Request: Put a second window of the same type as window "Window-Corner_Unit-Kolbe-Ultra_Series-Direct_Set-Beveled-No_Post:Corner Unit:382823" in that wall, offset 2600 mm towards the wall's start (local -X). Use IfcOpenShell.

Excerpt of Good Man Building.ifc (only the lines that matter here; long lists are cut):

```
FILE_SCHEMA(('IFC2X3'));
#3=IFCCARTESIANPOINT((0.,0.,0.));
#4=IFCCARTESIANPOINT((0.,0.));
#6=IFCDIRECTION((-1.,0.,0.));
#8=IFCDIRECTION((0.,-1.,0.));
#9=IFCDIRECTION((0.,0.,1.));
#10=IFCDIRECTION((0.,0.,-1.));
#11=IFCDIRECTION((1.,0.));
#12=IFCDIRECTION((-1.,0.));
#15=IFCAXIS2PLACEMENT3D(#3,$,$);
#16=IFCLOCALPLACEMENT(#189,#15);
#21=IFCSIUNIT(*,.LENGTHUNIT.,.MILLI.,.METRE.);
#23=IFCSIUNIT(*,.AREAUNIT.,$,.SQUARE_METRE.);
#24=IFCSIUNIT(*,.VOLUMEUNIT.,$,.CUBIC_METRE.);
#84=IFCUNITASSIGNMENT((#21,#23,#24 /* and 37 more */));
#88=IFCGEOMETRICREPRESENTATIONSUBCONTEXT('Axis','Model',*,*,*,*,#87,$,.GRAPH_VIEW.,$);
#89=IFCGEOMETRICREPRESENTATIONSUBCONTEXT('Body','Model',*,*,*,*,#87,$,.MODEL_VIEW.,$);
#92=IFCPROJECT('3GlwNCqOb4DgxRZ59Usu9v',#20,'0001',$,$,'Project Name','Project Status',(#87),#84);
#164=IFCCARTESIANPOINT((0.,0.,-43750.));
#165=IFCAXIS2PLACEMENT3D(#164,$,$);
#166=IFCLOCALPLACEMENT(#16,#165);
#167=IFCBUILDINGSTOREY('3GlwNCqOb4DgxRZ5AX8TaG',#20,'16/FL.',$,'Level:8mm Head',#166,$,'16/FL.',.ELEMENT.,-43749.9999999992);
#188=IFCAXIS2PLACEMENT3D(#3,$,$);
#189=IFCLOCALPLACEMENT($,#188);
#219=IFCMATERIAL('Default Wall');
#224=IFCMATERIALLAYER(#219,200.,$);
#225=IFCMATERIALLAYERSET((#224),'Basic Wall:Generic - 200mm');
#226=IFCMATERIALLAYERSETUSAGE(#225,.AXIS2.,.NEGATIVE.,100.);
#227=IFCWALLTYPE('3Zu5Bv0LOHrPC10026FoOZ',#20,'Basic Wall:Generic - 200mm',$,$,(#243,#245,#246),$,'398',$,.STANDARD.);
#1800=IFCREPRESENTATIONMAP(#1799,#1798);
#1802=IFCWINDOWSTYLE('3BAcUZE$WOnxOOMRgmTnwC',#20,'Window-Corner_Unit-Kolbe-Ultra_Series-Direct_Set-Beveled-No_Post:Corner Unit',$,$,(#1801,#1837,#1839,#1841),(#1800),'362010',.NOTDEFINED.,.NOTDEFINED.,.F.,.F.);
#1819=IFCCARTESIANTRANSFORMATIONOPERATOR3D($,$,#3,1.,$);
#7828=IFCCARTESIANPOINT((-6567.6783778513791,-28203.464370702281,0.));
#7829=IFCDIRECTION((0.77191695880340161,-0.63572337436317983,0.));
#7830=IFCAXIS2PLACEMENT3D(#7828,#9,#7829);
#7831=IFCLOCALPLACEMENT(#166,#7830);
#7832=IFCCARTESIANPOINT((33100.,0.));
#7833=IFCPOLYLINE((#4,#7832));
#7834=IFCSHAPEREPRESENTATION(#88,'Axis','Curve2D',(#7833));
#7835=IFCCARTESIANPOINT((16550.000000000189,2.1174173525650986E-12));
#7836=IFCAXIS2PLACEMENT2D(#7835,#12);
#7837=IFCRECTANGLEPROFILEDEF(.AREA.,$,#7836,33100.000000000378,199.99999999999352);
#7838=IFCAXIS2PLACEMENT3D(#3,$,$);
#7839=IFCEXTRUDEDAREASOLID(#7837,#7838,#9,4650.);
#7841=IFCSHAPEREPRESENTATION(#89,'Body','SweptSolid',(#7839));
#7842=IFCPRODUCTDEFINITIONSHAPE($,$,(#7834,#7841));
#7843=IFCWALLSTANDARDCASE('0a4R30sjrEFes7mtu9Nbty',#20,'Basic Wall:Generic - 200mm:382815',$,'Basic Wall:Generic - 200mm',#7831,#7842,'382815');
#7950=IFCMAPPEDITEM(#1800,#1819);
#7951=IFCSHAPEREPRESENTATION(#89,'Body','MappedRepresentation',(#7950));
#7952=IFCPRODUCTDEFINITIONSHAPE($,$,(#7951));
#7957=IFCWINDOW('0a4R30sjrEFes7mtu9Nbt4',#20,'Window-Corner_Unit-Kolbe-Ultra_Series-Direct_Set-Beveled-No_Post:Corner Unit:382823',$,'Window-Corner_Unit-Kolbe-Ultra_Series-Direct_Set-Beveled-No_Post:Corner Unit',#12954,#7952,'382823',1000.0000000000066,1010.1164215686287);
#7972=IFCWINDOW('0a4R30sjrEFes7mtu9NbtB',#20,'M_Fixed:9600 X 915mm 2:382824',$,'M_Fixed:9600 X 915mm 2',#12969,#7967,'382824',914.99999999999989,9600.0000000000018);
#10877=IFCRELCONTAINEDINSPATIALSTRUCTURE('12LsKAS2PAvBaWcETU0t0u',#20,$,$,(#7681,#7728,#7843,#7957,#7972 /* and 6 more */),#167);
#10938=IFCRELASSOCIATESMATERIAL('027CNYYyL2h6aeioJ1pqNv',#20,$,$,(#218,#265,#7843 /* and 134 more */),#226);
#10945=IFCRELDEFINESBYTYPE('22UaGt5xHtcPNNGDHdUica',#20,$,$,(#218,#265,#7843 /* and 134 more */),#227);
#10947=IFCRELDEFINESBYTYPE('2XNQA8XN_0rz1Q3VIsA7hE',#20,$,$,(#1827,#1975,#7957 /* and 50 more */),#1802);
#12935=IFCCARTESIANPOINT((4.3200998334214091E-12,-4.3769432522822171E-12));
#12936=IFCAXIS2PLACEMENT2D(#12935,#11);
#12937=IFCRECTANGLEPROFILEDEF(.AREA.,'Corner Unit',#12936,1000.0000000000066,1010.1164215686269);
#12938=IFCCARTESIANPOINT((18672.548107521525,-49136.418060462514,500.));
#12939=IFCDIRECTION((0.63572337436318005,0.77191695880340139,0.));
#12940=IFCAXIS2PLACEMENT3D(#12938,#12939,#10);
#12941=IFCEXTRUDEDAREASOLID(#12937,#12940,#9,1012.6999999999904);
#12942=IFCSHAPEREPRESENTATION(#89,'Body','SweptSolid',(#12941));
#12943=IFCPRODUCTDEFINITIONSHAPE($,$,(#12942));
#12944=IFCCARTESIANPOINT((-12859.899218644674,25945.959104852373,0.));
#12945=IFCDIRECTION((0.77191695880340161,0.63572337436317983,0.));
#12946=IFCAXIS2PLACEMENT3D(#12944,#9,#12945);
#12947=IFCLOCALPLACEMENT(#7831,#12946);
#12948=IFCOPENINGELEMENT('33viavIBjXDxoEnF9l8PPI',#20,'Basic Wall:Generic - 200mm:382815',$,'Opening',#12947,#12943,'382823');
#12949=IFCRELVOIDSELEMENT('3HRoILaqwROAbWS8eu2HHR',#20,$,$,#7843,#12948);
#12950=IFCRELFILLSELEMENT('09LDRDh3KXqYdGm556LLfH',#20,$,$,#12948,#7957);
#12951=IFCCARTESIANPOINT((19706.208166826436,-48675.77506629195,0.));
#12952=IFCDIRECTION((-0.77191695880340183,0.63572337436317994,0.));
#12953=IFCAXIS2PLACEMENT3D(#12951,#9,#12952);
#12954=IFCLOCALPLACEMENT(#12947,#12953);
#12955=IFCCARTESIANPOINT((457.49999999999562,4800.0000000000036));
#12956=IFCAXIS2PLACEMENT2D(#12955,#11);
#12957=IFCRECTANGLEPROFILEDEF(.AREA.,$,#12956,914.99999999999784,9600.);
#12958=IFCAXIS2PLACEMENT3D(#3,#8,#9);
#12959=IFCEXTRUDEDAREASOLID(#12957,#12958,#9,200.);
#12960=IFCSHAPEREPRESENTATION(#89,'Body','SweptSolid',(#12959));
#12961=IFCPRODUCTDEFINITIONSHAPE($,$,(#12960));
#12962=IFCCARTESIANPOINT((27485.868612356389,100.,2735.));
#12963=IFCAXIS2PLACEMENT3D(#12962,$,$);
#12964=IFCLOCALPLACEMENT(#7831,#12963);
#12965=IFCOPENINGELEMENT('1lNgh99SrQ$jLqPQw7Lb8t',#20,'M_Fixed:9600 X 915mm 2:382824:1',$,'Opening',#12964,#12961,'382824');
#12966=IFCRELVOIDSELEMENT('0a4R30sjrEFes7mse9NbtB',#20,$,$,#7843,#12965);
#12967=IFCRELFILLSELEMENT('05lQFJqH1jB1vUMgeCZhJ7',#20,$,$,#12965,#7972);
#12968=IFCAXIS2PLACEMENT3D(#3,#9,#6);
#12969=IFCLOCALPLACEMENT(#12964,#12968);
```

```python
import ifcopenshell
import ifcopenshell.api.feature
import ifcopenshell.api.geometry
import ifcopenshell.api.root
import ifcopenshell.geom
import ifcopenshell.util.element
import ifcopenshell.util.placement
import ifcopenshell.util.shape

model = ifcopenshell.open("Good Man Building.ifc")
settings = ifcopenshell.geom.settings()


def volume(element):
    """Net volume in cubic metres, openings subtracted."""
    shape = ifcopenshell.geom.create_shape(settings, element)
    return ifcopenshell.util.shape.get_volume(shape.geometry)


def reuse_history(source, copy):
    """copy_class also copies each property set's owner history, people and application; keep the originals."""
    for rel in copy.IsDefinedBy:
        if rel.is_a("IfcRelDefinesByProperties") and (history := rel.RelatingPropertyDefinition.OwnerHistory):
            rel.RelatingPropertyDefinition.OwnerHistory = source.OwnerHistory
            ifcopenshell.util.element.remove_deep2(model, history)


window = model.by_guid("0a4R30sjrEFes7mtu9Nbt4")
opening = window.FillsVoids[0].RelatingOpeningElement
wall = opening.VoidsElements[0].RelatingBuildingElement
before = volume(wall)
shift = ifcopenshell.util.placement.get_local_placement(wall.ObjectPlacement)[:3, 0] * -2600.0

# copy_class copies the void relationship, type, container and properties, but no geometry.
new_opening = ifcopenshell.api.root.copy_class(model, product=opening)
new_opening.Representation = ifcopenshell.util.element.copy_deep(
    model, opening.Representation, exclude=["IfcGeometricRepresentationContext", "IfcRepresentationMap"]
)
new_opening.Name = "Basic Wall:Generic - 200mm"
new_opening.Tag = None
new_window = ifcopenshell.api.root.copy_class(model, product=window)
new_window.Representation = ifcopenshell.util.element.copy_deep(
    model, window.Representation, exclude=["IfcGeometricRepresentationContext", "IfcRepresentationMap"]
)
new_window.Name = "Window-Corner_Unit-Kolbe-Ultra_Series-Direct_Set-Beveled-No_Post:Corner Unit"
new_window.Tag = None
reuse_history(window, new_window)
fills = ifcopenshell.api.feature.add_filling(model, opening=new_opening, element=new_window)
fills.OwnerHistory = new_window.OwnerHistory  # required in IFC2X3

for old, new in ((opening, new_opening), (window, new_window)):
    matrix = ifcopenshell.util.placement.get_local_placement(old.ObjectPlacement)
    matrix[:3, 3] += shift
    ifcopenshell.api.geometry.edit_object_placement(model, product=new, matrix=matrix, is_si=False)

after = volume(wall)

print(f"wall volume {before:.3f} -> {after:.3f} m3")

model.write("Good Man Building_edited.ifc")
```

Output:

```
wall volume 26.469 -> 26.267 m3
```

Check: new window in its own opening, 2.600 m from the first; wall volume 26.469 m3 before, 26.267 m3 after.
